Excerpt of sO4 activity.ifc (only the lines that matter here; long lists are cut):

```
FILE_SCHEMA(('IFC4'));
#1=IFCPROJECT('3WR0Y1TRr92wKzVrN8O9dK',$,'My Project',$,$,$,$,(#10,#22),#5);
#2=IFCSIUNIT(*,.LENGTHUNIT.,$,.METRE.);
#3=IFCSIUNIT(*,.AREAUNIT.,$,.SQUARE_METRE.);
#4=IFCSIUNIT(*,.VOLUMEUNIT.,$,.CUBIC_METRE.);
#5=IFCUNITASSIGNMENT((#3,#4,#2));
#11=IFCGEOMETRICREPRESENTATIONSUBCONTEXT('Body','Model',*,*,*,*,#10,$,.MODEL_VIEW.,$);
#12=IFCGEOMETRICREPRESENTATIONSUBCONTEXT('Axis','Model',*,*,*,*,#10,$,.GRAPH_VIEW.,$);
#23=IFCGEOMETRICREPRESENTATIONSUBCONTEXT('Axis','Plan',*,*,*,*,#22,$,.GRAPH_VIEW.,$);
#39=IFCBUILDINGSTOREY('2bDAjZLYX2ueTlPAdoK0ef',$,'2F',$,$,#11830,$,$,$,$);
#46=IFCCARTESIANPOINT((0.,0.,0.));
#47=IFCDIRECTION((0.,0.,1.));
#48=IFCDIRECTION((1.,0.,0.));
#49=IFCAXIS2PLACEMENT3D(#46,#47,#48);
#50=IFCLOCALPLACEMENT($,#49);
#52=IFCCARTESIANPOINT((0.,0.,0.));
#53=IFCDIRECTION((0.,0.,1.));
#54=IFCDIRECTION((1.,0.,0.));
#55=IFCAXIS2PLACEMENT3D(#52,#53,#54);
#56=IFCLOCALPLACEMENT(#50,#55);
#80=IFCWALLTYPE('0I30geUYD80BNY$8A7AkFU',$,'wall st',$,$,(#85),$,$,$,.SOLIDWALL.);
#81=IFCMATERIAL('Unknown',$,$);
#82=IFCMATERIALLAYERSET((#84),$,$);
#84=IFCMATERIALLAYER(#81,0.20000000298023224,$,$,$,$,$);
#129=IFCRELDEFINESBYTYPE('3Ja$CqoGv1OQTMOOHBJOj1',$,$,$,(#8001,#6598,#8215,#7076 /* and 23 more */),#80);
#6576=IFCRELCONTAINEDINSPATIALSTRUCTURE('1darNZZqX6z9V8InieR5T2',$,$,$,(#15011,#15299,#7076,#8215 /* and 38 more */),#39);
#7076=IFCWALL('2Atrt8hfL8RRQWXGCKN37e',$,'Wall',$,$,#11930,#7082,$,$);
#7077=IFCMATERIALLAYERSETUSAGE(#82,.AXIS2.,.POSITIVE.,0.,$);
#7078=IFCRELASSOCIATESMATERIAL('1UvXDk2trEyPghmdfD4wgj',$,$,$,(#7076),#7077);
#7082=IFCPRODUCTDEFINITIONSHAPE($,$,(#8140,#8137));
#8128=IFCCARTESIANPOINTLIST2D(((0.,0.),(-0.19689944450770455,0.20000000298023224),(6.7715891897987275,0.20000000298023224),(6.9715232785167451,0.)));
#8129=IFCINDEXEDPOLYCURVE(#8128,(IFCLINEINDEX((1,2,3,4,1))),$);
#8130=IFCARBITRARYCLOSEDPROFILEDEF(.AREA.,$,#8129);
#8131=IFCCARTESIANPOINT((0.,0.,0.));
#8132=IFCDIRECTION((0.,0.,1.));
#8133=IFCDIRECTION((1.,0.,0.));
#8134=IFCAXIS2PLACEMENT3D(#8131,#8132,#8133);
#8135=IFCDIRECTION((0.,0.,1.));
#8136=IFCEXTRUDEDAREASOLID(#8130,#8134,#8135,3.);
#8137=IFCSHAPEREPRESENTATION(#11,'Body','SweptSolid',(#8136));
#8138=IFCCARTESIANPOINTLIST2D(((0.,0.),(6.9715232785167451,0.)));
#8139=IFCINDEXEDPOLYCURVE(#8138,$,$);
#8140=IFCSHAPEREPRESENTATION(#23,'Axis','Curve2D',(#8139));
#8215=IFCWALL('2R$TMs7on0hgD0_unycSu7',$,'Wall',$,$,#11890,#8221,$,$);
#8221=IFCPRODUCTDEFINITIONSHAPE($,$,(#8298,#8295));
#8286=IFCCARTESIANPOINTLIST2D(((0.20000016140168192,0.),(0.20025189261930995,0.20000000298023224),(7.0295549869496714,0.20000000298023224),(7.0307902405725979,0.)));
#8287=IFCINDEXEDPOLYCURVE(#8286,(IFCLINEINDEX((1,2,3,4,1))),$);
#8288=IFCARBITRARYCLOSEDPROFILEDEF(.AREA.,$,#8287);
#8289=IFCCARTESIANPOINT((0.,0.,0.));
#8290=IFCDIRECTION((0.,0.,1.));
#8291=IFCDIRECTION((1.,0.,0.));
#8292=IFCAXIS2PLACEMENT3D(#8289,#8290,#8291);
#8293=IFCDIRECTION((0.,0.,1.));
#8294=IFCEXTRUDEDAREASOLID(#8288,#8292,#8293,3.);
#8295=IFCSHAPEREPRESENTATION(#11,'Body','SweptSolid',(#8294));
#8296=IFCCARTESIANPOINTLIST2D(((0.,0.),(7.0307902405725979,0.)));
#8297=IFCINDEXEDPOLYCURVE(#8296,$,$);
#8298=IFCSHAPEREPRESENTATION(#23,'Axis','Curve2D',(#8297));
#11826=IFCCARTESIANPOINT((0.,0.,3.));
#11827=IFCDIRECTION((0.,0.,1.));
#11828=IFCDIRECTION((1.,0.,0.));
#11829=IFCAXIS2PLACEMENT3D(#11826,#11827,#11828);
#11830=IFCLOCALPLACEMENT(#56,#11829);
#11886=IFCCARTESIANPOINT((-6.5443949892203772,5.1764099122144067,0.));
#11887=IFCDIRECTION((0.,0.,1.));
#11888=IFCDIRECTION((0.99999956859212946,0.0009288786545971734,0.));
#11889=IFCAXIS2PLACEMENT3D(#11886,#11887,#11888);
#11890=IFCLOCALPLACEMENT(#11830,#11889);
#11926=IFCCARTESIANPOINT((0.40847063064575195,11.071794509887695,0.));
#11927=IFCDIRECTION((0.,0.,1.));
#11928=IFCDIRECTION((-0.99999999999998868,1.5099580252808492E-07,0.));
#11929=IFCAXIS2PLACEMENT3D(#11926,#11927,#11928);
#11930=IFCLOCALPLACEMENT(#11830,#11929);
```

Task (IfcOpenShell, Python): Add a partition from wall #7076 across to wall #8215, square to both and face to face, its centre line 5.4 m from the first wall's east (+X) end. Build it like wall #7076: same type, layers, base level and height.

```python
import numpy as np
import ifcopenshell
import ifcopenshell.api.geometry
import ifcopenshell.api.material
import ifcopenshell.api.pset
import ifcopenshell.api.root
import ifcopenshell.api.spatial
import ifcopenshell.api.type
import ifcopenshell.geom
import ifcopenshell.util.element
import ifcopenshell.util.placement
import ifcopenshell.util.representation
import ifcopenshell.util.shape
import ifcopenshell.util.unit

model = ifcopenshell.open("sO4 activity.ifc")
unit_scale = ifcopenshell.util.unit.calculate_unit_scale(model)
settings = ifcopenshell.geom.settings()
settings.set("use-world-coords", True)

start_wall = model.by_id(7076)
end_wall = model.by_guid("2R$TMs7on0hgD0_unycSu7")
like = model.by_guid("2Atrt8hfL8RRQWXGCKN37e")
matrix = ifcopenshell.util.placement.get_local_placement(start_wall.ObjectPlacement)
matrix[:3, 3] *= unit_scale


def extent(element):
    """Bounding box in the first wall's axes, in metres."""
    shape = ifcopenshell.geom.create_shape(settings, element)
    points = (ifcopenshell.util.shape.get_vertices(shape.geometry) - matrix[:3, 3]) @ matrix[:3, :3]
    return points.min(axis=0), points.max(axis=0)


y_start = extent(start_wall)[1][1]
y_end = extent(end_wall)[0][1]
like_min, like_max = extent(like)
length, height = float(abs(y_end - y_start)), float(like_max[2] - like_min[2])
layer_set = ifcopenshell.util.element.get_material(like, should_skip_usage=True)
thickness = sum(layer.LayerThickness for layer in layer_set.MaterialLayers) * unit_scale

wall = ifcopenshell.api.root.create_entity(model, ifc_class="IfcWall", name="New partition")
storey = ifcopenshell.util.element.get_container(like)
ifcopenshell.api.spatial.assign_container(model, products=[wall], relating_structure=storey)
ifcopenshell.api.type.assign_type(
    model, related_objects=[wall], relating_type=ifcopenshell.util.element.get_type(like), should_map_representations=False
)
rel = ifcopenshell.api.material.assign_material(
    model, products=[wall], type="IfcMaterialLayerSetUsage", material=layer_set
)
rel.RelatingMaterial.OffsetFromReferenceLine = -thickness / 2 / unit_scale
pset = ifcopenshell.api.pset.add_pset(model, product=wall, name="Pset_WallCommon")
ifcopenshell.api.pset.edit_pset(model, pset=pset, properties={"IsExternal": False, "LoadBearing": False})

# The axis runs down the middle of the wall.
axis = ifcopenshell.api.geometry.add_axis_representation(
    model, context=ifcopenshell.util.representation.get_context(model, "Model", "Axis"), axis=[(0.0, 0.0), (length, 0.0)]
)
body = ifcopenshell.api.geometry.add_wall_representation(
    model,
    context=ifcopenshell.util.representation.get_context(model, "Model", "Body", "MODEL_VIEW"),
    length=length,
    height=height,
    thickness=thickness,
    offset=-thickness / 2,
)
for representation in (axis, body):
    ifcopenshell.api.geometry.assign_representation(model, product=wall, representation=representation)

placement = matrix @ ifcopenshell.util.placement.rotation(90, "Z")
placement[:, 3] = matrix @ np.array([extent(start_wall)[0][0] + 5.4, y_start, like_min[2], 1.0])
ifcopenshell.api.geometry.edit_object_placement(model, product=wall, matrix=placement)

print(f"partition {length:.3f} m long, {height:.3f} m high, {thickness:.3f} m thick")

model.write("sO4 activity_rev.ifc")
```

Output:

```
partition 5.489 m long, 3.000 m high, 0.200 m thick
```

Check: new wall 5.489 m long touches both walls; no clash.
